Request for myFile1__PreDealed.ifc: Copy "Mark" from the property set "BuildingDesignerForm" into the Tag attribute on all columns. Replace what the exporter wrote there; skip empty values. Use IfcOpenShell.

First a look at what the model holds.

```python
import ifcopenshell
import ifcopenshell.util.element

model = ifcopenshell.open("myFile1__PreDealed.ifc")
print(model.schema)
columns = model.by_type("IfcColumn")
print(len(columns), "columns")
for e in columns[:8]:
    source = ifcopenshell.util.element.get_pset(e, "BuildingDesignerForm", "Mark")
    target = e.Tag
    print(e.id(), repr(source), repr(target), sep=" | ")
```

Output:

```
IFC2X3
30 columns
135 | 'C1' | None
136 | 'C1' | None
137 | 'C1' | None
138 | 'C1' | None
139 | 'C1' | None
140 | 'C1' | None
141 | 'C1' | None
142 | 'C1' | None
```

```python
import ifcopenshell
import ifcopenshell.util.element

model = ifcopenshell.open("myFile1__PreDealed.ifc")

count = 0
for e in model.by_type("IfcColumn"):
    value = ifcopenshell.util.element.get_pset(e, "BuildingDesignerForm", "Mark")
    current = e.Tag
    if not value or not value.strip() or current == value:
        continue
    e.Tag = value
    count += 1

print(count, "columns updated")

model.write("myFile1__PreDealed_updated.ifc")
```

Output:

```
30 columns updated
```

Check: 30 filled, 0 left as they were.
